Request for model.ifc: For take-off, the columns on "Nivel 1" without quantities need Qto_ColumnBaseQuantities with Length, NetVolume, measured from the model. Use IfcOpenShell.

First a look at what the model holds.

```python
import ifcopenshell
import ifcopenshell.util.element
import ifcopenshell.util.unit

model = ifcopenshell.open("model.ifc")
print(model.schema)
for unit_type in ("LENGTHUNIT", "AREAUNIT", "VOLUMEUNIT"):
    print(unit_type, ifcopenshell.util.unit.calculate_unit_scale(model, unit_type))
storey = next(s for s in model.by_type("IfcBuildingStorey") if s.Name == "Nivel 1")
columns = [e for e in ifcopenshell.util.element.get_decomposition(storey) if e.is_a("IfcColumn")]
for e in sorted(columns, key=lambda e: e.id()):
    print(e.id(), e.is_a(), e.Name, list(ifcopenshell.util.element.get_psets(e, qtos_only=True)), sep=" | ")
```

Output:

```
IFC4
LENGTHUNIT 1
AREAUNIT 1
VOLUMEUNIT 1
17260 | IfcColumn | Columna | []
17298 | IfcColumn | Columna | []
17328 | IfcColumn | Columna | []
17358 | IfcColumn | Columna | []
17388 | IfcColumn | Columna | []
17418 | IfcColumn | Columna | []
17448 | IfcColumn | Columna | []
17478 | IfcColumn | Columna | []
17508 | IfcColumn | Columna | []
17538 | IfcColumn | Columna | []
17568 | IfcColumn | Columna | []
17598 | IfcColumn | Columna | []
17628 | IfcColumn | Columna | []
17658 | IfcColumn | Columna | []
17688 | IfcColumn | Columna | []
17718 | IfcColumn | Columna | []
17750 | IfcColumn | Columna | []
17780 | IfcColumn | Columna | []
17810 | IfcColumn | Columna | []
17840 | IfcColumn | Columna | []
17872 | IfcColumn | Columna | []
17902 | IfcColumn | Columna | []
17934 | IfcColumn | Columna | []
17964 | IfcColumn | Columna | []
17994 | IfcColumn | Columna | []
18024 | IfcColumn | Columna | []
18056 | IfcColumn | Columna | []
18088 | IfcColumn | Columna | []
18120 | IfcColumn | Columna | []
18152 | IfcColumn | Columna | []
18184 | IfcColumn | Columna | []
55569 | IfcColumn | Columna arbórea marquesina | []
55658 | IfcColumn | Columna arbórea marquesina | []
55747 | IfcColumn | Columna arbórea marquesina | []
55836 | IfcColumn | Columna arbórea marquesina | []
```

```python
import ifcopenshell
import ifcopenshell.api.pset
import ifcopenshell.geom
import ifcopenshell.util.element
import ifcopenshell.util.shape
import ifcopenshell.util.unit

model = ifcopenshell.open("model.ifc")
unit_scale = ifcopenshell.util.unit.calculate_unit_scale(model)
volume_scale = ifcopenshell.util.unit.calculate_unit_scale(model, "VOLUMEUNIT")
settings = ifcopenshell.geom.settings()

storey = next(s for s in model.by_type("IfcBuildingStorey") if s.Name == "Nivel 1")
columns = [e for e in ifcopenshell.util.element.get_decomposition(storey) if e.is_a("IfcColumn")]

for e in sorted(columns, key=lambda e: e.id()):
    if ifcopenshell.util.element.get_psets(e, qtos_only=True, should_inherit=False):
        continue
    # Geometry comes back in metres, in the element's own axes.
    shape = ifcopenshell.geom.create_shape(settings, e)
    values = {
        "Length": ifcopenshell.util.shape.get_z(shape.geometry) / unit_scale,
        "NetVolume": ifcopenshell.util.shape.get_volume(shape.geometry) / volume_scale,
    }
    qto = ifcopenshell.api.pset.add_qto(model, product=e, name="Qto_ColumnBaseQuantities")
    ifcopenshell.api.pset.edit_qto(model, qto=qto, properties=values)
    print(e.id(), {k: round(v, 3) for k, v in values.items()})

model.write("model_edited.ifc")
```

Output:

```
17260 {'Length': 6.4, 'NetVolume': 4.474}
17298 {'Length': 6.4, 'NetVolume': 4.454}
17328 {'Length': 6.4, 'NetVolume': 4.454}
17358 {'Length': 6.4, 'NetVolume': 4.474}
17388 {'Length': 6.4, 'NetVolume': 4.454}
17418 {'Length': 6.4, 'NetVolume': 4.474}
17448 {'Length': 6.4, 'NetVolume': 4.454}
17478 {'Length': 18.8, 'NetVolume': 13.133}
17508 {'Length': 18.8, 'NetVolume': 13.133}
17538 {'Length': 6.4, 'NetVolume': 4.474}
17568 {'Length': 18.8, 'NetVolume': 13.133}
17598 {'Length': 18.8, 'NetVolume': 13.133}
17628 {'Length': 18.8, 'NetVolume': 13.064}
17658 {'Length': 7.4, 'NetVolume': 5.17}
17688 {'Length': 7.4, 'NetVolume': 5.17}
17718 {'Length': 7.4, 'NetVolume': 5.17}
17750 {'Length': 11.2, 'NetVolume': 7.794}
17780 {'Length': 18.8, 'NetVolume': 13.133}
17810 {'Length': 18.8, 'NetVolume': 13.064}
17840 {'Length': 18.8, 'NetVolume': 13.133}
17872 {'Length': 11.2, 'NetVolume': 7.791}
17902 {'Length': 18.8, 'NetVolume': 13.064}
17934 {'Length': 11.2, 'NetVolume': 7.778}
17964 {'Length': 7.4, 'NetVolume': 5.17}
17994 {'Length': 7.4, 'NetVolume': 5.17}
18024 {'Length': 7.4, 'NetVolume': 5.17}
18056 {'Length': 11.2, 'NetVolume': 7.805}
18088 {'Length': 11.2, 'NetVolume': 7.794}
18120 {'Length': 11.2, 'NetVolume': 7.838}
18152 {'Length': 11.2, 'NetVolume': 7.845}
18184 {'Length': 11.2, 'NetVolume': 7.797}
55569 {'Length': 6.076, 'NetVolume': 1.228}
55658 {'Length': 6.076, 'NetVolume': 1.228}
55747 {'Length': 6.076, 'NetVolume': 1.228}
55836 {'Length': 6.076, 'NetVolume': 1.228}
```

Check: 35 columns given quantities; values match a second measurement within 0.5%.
